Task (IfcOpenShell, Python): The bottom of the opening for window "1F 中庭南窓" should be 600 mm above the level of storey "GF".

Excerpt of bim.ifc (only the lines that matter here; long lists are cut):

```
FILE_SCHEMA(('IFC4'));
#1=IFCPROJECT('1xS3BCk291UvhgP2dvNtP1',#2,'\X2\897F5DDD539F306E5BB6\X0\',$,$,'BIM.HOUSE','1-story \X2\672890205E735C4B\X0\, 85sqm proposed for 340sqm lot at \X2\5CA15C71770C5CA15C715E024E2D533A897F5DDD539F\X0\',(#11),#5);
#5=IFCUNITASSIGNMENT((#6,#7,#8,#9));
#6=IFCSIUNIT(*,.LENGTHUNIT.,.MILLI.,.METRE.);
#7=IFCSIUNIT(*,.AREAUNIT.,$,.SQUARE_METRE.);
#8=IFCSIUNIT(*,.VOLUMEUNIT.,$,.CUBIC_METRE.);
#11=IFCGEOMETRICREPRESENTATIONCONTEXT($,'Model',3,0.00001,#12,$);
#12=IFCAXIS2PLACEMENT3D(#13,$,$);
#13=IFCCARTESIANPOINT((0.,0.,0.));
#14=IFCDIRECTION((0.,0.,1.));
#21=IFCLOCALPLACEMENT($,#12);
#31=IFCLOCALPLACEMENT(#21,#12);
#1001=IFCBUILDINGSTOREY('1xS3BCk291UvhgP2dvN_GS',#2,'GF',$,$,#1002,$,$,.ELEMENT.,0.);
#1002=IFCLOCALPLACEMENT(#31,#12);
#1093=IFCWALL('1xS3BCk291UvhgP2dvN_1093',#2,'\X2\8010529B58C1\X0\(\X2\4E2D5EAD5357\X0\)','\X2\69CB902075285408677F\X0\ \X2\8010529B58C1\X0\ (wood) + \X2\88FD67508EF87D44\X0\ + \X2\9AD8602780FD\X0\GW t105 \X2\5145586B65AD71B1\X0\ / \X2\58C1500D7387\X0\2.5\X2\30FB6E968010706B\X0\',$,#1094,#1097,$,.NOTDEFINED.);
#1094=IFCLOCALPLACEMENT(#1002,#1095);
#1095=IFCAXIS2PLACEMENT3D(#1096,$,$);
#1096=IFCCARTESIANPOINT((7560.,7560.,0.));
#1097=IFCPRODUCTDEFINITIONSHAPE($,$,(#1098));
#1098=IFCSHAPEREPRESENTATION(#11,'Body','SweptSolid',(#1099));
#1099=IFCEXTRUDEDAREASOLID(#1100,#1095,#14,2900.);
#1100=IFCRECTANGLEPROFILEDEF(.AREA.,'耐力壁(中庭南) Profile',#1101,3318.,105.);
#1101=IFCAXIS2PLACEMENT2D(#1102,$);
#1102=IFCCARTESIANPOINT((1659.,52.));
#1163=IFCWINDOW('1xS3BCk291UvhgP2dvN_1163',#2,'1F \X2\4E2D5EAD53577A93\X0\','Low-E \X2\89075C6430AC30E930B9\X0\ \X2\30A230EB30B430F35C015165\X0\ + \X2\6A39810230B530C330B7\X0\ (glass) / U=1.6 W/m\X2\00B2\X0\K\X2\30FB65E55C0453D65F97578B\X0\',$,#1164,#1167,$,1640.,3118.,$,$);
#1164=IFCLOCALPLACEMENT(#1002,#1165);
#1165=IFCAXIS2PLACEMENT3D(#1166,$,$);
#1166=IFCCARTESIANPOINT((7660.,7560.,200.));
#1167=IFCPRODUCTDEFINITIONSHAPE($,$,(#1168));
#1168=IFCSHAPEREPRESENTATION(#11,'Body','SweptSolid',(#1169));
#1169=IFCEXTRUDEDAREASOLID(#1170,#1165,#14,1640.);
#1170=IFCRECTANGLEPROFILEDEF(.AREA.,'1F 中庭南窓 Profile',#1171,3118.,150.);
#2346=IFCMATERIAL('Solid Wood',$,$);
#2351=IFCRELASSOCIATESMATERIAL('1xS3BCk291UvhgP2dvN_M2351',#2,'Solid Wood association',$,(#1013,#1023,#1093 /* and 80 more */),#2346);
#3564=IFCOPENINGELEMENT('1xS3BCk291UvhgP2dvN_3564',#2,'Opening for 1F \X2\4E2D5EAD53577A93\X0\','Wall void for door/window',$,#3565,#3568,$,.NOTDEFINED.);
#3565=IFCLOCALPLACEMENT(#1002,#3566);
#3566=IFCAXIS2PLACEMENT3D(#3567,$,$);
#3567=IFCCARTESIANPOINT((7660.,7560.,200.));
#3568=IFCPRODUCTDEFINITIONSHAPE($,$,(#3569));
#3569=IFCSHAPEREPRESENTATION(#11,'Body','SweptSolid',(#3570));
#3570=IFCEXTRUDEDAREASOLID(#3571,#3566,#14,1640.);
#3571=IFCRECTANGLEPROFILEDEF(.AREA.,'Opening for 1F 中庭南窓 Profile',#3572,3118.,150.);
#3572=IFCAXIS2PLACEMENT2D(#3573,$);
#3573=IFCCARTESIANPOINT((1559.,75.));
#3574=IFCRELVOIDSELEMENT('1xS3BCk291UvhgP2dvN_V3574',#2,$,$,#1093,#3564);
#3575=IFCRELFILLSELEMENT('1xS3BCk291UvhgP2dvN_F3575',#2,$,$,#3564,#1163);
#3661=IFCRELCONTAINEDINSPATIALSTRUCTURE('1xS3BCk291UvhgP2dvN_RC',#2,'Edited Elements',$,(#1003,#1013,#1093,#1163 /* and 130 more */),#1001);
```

```python
import numpy as np
import ifcopenshell
import ifcopenshell.api.geometry
import ifcopenshell.geom
import ifcopenshell.util.element
import ifcopenshell.util.placement
import ifcopenshell.util.shape
import ifcopenshell.util.unit

model = ifcopenshell.open("bim.ifc")
unit_scale = ifcopenshell.util.unit.calculate_unit_scale(model)

window = model.by_guid("1xS3BCk291UvhgP2dvN_1163")
opening = window.FillsVoids[0].RelatingOpeningElement
storey = ifcopenshell.util.element.get_container(window, ifc_class="IfcBuildingStorey")
level = ifcopenshell.util.placement.get_local_placement(storey.ObjectPlacement)[2, 3]

# The opening's origin need not be at the sill, so measure its lowest point.
shape = ifcopenshell.geom.create_shape(ifcopenshell.geom.settings(), opening)
bottom = ifcopenshell.util.shape.get_shape_bottom_elevation(shape, shape.geometry) / unit_scale
dz = level + 600.0 - bottom

shift = np.array([0.0, 0.0, dz])
# The window is not placed relative to its opening, so move both.
for product in (opening, window):
    matrix = ifcopenshell.util.placement.get_local_placement(product.ObjectPlacement)
    matrix[:3, 3] += shift
    ifcopenshell.api.geometry.edit_object_placement(model, product=product, matrix=matrix, is_si=False)

print(f"moved by {dz * unit_scale:+.3f} m")

model.write("bim-out.ifc")
```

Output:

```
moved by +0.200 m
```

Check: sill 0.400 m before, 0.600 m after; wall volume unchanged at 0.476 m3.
